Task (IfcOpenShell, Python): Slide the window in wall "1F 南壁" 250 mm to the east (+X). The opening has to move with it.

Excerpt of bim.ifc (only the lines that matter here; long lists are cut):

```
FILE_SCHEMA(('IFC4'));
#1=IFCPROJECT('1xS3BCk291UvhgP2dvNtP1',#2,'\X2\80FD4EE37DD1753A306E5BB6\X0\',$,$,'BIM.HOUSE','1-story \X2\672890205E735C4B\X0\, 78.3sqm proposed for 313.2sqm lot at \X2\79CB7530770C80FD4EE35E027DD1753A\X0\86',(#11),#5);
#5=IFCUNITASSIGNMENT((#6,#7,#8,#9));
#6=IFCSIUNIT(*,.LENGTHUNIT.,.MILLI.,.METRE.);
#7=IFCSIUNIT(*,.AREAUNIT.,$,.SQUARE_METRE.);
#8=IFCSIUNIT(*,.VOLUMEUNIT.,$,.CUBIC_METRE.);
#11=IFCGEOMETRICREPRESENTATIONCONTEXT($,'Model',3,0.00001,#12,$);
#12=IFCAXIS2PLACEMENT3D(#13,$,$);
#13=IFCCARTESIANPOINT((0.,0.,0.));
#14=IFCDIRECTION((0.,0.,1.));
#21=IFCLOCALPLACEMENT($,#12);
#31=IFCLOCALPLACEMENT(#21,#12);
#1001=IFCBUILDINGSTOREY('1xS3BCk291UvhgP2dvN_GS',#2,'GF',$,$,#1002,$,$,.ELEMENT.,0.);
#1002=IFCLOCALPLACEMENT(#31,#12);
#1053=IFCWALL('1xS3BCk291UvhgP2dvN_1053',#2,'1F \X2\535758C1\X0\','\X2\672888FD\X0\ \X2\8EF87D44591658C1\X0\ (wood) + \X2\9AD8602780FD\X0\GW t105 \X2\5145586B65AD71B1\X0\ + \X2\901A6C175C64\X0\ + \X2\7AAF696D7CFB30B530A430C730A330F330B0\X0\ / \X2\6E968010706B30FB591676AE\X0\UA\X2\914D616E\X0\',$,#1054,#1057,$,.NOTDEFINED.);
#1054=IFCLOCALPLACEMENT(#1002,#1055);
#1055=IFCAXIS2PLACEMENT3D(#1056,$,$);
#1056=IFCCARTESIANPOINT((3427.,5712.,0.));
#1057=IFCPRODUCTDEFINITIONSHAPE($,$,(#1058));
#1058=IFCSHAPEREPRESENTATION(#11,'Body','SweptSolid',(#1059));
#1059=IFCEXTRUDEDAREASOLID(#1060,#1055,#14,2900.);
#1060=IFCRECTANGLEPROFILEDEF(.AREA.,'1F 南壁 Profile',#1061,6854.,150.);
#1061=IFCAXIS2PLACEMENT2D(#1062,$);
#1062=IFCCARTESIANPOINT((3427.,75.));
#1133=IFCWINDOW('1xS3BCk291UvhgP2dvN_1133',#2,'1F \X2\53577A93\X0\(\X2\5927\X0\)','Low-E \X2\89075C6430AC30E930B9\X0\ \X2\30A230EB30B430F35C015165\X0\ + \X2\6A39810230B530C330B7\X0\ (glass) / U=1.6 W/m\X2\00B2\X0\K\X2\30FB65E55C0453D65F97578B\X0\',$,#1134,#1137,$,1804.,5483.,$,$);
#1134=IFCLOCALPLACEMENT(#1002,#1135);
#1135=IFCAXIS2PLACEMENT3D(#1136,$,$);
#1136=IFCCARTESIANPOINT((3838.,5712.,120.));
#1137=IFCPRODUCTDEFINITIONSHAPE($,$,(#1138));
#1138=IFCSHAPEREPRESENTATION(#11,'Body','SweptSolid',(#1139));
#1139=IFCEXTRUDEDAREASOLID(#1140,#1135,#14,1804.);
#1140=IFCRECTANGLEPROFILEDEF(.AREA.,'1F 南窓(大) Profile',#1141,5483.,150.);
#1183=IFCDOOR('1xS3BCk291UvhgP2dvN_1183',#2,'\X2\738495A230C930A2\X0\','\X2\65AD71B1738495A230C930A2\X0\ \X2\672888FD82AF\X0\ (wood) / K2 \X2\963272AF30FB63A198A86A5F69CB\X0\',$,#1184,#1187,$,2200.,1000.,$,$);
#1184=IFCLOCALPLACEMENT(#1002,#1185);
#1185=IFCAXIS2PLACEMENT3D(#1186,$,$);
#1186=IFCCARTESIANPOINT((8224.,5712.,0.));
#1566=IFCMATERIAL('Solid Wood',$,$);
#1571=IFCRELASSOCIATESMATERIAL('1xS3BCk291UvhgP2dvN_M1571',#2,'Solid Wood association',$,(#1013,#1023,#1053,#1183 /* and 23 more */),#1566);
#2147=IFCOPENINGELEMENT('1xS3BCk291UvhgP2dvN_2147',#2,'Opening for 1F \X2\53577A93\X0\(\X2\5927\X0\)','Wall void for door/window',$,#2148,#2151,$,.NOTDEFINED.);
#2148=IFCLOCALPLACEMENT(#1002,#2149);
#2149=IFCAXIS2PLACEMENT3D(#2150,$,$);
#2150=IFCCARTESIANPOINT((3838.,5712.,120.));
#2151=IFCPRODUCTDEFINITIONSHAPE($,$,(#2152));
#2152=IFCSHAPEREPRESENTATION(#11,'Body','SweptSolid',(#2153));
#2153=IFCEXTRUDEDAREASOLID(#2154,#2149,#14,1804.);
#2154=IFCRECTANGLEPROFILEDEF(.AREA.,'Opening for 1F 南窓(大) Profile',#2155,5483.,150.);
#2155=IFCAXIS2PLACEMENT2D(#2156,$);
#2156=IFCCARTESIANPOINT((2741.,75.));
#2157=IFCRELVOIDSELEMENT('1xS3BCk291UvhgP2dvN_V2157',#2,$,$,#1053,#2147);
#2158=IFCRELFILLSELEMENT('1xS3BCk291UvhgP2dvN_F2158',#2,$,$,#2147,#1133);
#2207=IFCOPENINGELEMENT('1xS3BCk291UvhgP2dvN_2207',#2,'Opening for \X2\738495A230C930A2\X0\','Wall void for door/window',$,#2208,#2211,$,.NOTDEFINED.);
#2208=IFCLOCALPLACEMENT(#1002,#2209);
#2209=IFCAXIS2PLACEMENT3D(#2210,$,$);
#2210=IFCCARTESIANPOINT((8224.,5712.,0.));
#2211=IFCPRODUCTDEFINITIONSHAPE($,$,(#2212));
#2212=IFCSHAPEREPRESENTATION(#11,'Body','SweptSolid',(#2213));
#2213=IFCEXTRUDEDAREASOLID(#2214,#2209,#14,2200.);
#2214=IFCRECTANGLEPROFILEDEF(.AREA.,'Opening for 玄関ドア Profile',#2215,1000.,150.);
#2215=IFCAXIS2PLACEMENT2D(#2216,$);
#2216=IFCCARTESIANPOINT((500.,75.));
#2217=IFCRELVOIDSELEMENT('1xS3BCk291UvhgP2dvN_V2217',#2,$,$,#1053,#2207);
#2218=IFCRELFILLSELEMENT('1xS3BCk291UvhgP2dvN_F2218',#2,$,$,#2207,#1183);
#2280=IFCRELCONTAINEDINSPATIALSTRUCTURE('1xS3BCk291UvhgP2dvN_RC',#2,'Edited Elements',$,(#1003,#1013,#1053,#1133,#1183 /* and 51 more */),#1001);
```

```python
import ifcopenshell
import ifcopenshell.api.geometry
import ifcopenshell.util.placement
import ifcopenshell.util.unit

model = ifcopenshell.open("bim.ifc")
unit_scale = ifcopenshell.util.unit.calculate_unit_scale(model)

window = model.by_id(1133)
opening = window.FillsVoids[0].RelatingOpeningElement
wall = opening.VoidsElements[0].RelatingBuildingElement

wall_matrix = ifcopenshell.util.placement.get_local_placement(wall.ObjectPlacement)
shift = wall_matrix[:3, 0] * 0.25 / unit_scale
before = ifcopenshell.util.placement.get_local_placement(window.ObjectPlacement)[:3, 3].copy()

# The window is not placed relative to its opening, so move both.
for product in (opening, window):
    matrix = ifcopenshell.util.placement.get_local_placement(product.ObjectPlacement)
    matrix[:3, 3] += shift
    ifcopenshell.api.geometry.edit_object_placement(model, product=product, matrix=matrix, is_si=False)

after = ifcopenshell.util.placement.get_local_placement(window.ObjectPlacement)[:3, 3]
print("window moved by", (after - before).round(3) + 0.0)

model.write("bim_rev.ifc")
```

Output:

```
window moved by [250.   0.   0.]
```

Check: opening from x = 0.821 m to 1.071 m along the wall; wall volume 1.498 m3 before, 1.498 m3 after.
